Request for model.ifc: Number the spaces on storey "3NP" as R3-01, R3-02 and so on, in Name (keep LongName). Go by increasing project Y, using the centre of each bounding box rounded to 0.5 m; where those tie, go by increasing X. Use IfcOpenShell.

First a look at what the model holds.

```python
import ifcopenshell
import ifcopenshell.util.element
import ifcopenshell.util.placement

model = ifcopenshell.open("model.ifc")
print(model.schema)
storey = next(s for s in model.by_type("IfcBuildingStorey") if s.Name == "3NP")
spaces = [e for e in ifcopenshell.util.element.get_decomposition(storey) if e.is_a("IfcSpace")]
for e in sorted(spaces, key=lambda e: e.id()):
    origin = ifcopenshell.util.placement.get_local_placement(e.ObjectPlacement)[:3, 3]
    print(e.id(), e.Name, e.LongName, origin.round(2) + 0.0, sep=" | ")
```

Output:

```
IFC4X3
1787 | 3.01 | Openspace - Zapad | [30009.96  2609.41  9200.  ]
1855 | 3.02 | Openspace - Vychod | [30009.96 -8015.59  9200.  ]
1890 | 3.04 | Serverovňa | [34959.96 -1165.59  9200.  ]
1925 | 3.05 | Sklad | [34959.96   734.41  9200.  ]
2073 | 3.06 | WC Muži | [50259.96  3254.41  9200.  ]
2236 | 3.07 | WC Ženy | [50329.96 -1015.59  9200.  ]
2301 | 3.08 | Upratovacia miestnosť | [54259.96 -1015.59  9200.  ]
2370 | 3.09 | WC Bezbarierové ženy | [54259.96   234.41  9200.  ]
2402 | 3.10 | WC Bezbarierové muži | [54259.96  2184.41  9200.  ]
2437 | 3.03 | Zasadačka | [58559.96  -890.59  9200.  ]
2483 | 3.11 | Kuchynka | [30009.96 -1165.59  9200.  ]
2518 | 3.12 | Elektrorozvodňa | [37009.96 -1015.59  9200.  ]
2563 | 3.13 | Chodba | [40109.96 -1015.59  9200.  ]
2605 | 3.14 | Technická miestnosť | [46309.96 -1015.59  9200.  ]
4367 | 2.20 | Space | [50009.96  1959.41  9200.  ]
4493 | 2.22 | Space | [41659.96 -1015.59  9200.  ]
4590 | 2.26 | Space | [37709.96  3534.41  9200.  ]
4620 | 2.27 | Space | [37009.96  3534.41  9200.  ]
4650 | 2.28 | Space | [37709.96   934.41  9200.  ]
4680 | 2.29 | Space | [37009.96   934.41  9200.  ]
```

```python
import ifcopenshell
import ifcopenshell.geom
import ifcopenshell.util.element
import ifcopenshell.util.shape

model = ifcopenshell.open("model.ifc")
settings = ifcopenshell.geom.settings()
settings.set("use-world-coords", True)


def centre(element):
    shape = ifcopenshell.geom.create_shape(settings, element)
    return ifcopenshell.util.shape.get_bbox_centroid(shape.geometry)


storey = next(s for s in model.by_type("IfcBuildingStorey") if s.Name == "3NP")
spaces = [e for e in ifcopenshell.util.element.get_decomposition(storey) if e.is_a("IfcSpace")]

# Insertion points can sit at a corner or the storey origin, so sort by the geometry (in metres).
centres = {e: centre(e) for e in spaces}
spaces.sort(key=lambda e: (round(centres[e][1] / 0.5), centres[e][0]))

for i, e in enumerate(spaces, start=1):
    number = f"R3-{i:02d}"
    e.Name = number
    print(e.id(), number)

model.write("model-out.ifc")
```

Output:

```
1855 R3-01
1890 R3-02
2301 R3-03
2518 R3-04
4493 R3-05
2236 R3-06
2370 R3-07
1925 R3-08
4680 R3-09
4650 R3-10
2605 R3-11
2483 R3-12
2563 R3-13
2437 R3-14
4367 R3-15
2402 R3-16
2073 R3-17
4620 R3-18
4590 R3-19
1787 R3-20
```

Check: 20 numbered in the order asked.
